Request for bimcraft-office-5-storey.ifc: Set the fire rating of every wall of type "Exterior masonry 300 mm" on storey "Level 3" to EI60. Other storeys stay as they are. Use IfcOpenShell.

First a look at what the model holds.

```python
import ifcopenshell
import ifcopenshell.util.element

model = ifcopenshell.open("bimcraft-office-5-storey.ifc")
print(model.schema)
storey = next(s for s in model.by_type("IfcBuildingStorey") if s.Name == "Level 3")
walls = [e for e in ifcopenshell.util.element.get_decomposition(storey) if e.is_a("IfcWall")]
seen = {}
for e in walls:
    element_type = ifcopenshell.util.element.get_type(e)
    key = (element_type.Name if element_type != e and element_type else None, ifcopenshell.util.element.get_pset(e, "Pset_WallCommon", "FireRating"))
    seen[key] = seen.get(key, 0) + 1
for (name, value), count in sorted(seen.items(), key=str):
    print(count, "x", name, "|", value)
```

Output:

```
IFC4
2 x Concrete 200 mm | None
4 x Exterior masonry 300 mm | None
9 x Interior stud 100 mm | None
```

```python
import ifcopenshell
import ifcopenshell.api.pset
import ifcopenshell.util.element

model = ifcopenshell.open("bimcraft-office-5-storey.ifc")

storey = next(s for s in model.by_type("IfcBuildingStorey") if s.Name == "Level 3")
walls = [e for e in ifcopenshell.util.element.get_decomposition(storey) if e.is_a("IfcWall")]

count = 0
for e in walls:
    element_type = ifcopenshell.util.element.get_type(e)
    if element_type in (None, e) or element_type.Name != "Exterior masonry 300 mm":
        continue
    # add_pset returns the element's existing set when there is one.
    pset = ifcopenshell.api.pset.add_pset(model, product=e, name="Pset_WallCommon")
    ifcopenshell.api.pset.edit_pset(model, pset=pset, properties={"FireRating": "EI60"})
    count += 1

print(count, "walls updated")

model.write("bimcraft-office-5-storey_rev.ifc")
```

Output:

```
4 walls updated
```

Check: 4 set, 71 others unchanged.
